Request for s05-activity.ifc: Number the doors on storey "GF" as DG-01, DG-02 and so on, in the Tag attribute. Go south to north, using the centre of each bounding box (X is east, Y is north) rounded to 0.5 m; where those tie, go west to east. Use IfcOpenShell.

First a look at what the model holds.

```python
import ifcopenshell
import ifcopenshell.util.element
import ifcopenshell.util.placement

model = ifcopenshell.open("s05-activity.ifc")
print(model.schema)
storey = next(s for s in model.by_type("IfcBuildingStorey") if s.Name == "GF")
doors = [e for e in ifcopenshell.util.element.get_decomposition(storey) if e.is_a("IfcDoor")]
for e in sorted(doors, key=lambda e: e.id()):
    origin = ifcopenshell.util.placement.get_local_placement(e.ObjectPlacement)[:3, 3]
    print(e.id(), e.Tag, e.Name, origin.round(2) + 0.0, sep=" | ")
```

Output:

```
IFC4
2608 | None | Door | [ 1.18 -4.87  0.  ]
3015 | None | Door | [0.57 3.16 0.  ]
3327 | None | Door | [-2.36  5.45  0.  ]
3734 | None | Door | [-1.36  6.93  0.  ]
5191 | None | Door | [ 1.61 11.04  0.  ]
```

```python
import ifcopenshell
import ifcopenshell.geom
import ifcopenshell.util.element
import ifcopenshell.util.shape

model = ifcopenshell.open("s05-activity.ifc")
settings = ifcopenshell.geom.settings()
settings.set("use-world-coords", True)


def centre(element):
    shape = ifcopenshell.geom.create_shape(settings, element)
    return ifcopenshell.util.shape.get_bbox_centroid(shape.geometry)


storey = next(s for s in model.by_type("IfcBuildingStorey") if s.Name == "GF")
doors = [e for e in ifcopenshell.util.element.get_decomposition(storey) if e.is_a("IfcDoor")]

# Insertion points can sit at a corner or the storey origin, so sort by the geometry (in metres).
centres = {e: centre(e) for e in doors}
doors.sort(key=lambda e: (round(centres[e][1] / 0.5), centres[e][0]))

for i, e in enumerate(doors, start=1):
    number = f"DG-{i:02d}"
    e.Tag = number
    print(e.id(), number)

model.write("s05-activity_rev.ifc")
```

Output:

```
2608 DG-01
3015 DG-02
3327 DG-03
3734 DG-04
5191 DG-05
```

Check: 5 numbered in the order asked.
